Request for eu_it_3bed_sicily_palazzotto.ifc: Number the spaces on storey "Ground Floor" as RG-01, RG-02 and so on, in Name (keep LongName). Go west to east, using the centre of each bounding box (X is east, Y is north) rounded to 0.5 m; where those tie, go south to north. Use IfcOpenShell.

First a look at what the model holds.

```python
import ifcopenshell
import ifcopenshell.util.element
import ifcopenshell.util.placement

model = ifcopenshell.open("eu_it_3bed_sicily_palazzotto.ifc")
print(model.schema)
storey = next(s for s in model.by_type("IfcBuildingStorey") if s.Name == "Ground Floor")
spaces = [e for e in ifcopenshell.util.element.get_decomposition(storey) if e.is_a("IfcSpace")]
for e in sorted(spaces, key=lambda e: e.id()):
    origin = ifcopenshell.util.placement.get_local_placement(e.ObjectPlacement)[:3, 3]
    print(e.id(), e.Name, e.LongName, origin.round(2) + 0.0, sep=" | ")
```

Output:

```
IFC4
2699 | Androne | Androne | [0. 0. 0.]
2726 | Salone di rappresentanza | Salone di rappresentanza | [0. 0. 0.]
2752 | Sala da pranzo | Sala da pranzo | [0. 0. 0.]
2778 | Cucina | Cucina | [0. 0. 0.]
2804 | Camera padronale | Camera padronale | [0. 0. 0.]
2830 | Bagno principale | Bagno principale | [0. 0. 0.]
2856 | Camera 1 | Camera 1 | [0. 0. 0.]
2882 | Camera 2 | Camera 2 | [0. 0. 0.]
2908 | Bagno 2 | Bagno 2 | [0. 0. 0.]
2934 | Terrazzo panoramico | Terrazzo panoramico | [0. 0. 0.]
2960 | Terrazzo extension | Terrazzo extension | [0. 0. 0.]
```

```python
import ifcopenshell
import ifcopenshell.geom
import ifcopenshell.util.element
import ifcopenshell.util.shape

model = ifcopenshell.open("eu_it_3bed_sicily_palazzotto.ifc")
settings = ifcopenshell.geom.settings()
settings.set("use-world-coords", True)


def centre(element):
    shape = ifcopenshell.geom.create_shape(settings, element)
    return ifcopenshell.util.shape.get_bbox_centroid(shape.geometry)


storey = next(s for s in model.by_type("IfcBuildingStorey") if s.Name == "Ground Floor")
spaces = [e for e in ifcopenshell.util.element.get_decomposition(storey) if e.is_a("IfcSpace")]

# Insertion points can sit at a corner or the storey origin, so sort by the geometry (in metres).
centres = {e: centre(e) for e in spaces}
spaces.sort(key=lambda e: (round(centres[e][0] / 0.5), centres[e][1]))

for i, e in enumerate(spaces, start=1):
    number = f"RG-{i:02d}"
    e.Name = number
    print(e.id(), number)

model.write("eu_it_3bed_sicily_palazzotto-out.ifc")
```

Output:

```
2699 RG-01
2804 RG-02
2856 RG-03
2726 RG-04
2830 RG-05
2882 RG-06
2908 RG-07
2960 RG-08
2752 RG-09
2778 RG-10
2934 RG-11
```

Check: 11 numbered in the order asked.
